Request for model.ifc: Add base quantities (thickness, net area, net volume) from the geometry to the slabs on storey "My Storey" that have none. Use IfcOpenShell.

First a look at what the model holds.

```python
import ifcopenshell
import ifcopenshell.util.element
import ifcopenshell.util.unit

model = ifcopenshell.open("model.ifc")
print(model.schema)
for unit_type in ("LENGTHUNIT", "AREAUNIT", "VOLUMEUNIT"):
    print(unit_type, ifcopenshell.util.unit.calculate_unit_scale(model, unit_type))
storey = next(s for s in model.by_type("IfcBuildingStorey") if s.Name == "My Storey")
slabs = [e for e in ifcopenshell.util.element.get_decomposition(storey) if e.is_a("IfcSlab")]
for e in sorted(slabs, key=lambda e: e.id()):
    print(e.id(), e.is_a(), e.Name, list(ifcopenshell.util.element.get_psets(e, qtos_only=True)), sep=" | ")
```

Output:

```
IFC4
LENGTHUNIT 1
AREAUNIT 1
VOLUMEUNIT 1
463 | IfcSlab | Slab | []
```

```python
import ifcopenshell
import ifcopenshell.api.pset
import ifcopenshell.geom
import ifcopenshell.util.element
import ifcopenshell.util.shape
import ifcopenshell.util.unit

model = ifcopenshell.open("model.ifc")
unit_scale = ifcopenshell.util.unit.calculate_unit_scale(model)
area_scale = ifcopenshell.util.unit.calculate_unit_scale(model, "AREAUNIT")
volume_scale = ifcopenshell.util.unit.calculate_unit_scale(model, "VOLUMEUNIT")
settings = ifcopenshell.geom.settings()

storey = next(s for s in model.by_type("IfcBuildingStorey") if s.Name == "My Storey")
slabs = [e for e in ifcopenshell.util.element.get_decomposition(storey) if e.is_a("IfcSlab")]

for e in sorted(slabs, key=lambda e: e.id()):
    if ifcopenshell.util.element.get_psets(e, qtos_only=True, should_inherit=False):
        continue
    # Geometry comes back in metres, in the element's own axes.
    shape = ifcopenshell.geom.create_shape(settings, e)
    values = {
        "Width": ifcopenshell.util.shape.get_z(shape.geometry) / unit_scale,
        "NetArea": ifcopenshell.util.shape.get_footprint_area(shape.geometry) / area_scale,
        "NetVolume": ifcopenshell.util.shape.get_volume(shape.geometry) / volume_scale,
    }
    qto = ifcopenshell.api.pset.add_qto(model, product=e, name="Qto_SlabBaseQuantities")
    ifcopenshell.api.pset.edit_qto(model, qto=qto, properties=values)
    print(e.id(), {k: round(v, 3) for k, v in values.items()})

model.write("model-out.ifc")
```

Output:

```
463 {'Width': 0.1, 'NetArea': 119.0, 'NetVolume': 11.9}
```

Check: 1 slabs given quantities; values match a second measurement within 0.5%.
